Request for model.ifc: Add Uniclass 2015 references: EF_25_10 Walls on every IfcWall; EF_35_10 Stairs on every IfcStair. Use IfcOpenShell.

First a look at what the model holds.

```python
import ifcopenshell

model = ifcopenshell.open("model.ifc")
print(model.schema)
print("classifications:", [c.Name for c in model.by_type("IfcClassification")])
for ifc_class in ("IfcDoor", "IfcRoof", "IfcStair", "IfcWall", "IfcWindow"):
    print(ifc_class, len(model.by_type(ifc_class)))
```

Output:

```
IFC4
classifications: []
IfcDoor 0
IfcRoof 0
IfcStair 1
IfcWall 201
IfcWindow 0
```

```python
import ifcopenshell
import ifcopenshell.api.classification

model = ifcopenshell.open("model.ifc")

system = ifcopenshell.api.classification.add_classification(model, classification="Uniclass 2015")

codes = {
    "IfcWall": ("EF_25_10", "Walls"),
    "IfcStair": ("EF_35_10", "Stairs"),
}
for ifc_class, (code, name) in codes.items():
    products = model.by_type(ifc_class)
    ifcopenshell.api.classification.add_reference(
        model, products=products, classification=system, identification=code, name=name
    )
    print(code, len(products))

model.write("model_v2.ifc")
```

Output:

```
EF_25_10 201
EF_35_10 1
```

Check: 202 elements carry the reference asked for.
